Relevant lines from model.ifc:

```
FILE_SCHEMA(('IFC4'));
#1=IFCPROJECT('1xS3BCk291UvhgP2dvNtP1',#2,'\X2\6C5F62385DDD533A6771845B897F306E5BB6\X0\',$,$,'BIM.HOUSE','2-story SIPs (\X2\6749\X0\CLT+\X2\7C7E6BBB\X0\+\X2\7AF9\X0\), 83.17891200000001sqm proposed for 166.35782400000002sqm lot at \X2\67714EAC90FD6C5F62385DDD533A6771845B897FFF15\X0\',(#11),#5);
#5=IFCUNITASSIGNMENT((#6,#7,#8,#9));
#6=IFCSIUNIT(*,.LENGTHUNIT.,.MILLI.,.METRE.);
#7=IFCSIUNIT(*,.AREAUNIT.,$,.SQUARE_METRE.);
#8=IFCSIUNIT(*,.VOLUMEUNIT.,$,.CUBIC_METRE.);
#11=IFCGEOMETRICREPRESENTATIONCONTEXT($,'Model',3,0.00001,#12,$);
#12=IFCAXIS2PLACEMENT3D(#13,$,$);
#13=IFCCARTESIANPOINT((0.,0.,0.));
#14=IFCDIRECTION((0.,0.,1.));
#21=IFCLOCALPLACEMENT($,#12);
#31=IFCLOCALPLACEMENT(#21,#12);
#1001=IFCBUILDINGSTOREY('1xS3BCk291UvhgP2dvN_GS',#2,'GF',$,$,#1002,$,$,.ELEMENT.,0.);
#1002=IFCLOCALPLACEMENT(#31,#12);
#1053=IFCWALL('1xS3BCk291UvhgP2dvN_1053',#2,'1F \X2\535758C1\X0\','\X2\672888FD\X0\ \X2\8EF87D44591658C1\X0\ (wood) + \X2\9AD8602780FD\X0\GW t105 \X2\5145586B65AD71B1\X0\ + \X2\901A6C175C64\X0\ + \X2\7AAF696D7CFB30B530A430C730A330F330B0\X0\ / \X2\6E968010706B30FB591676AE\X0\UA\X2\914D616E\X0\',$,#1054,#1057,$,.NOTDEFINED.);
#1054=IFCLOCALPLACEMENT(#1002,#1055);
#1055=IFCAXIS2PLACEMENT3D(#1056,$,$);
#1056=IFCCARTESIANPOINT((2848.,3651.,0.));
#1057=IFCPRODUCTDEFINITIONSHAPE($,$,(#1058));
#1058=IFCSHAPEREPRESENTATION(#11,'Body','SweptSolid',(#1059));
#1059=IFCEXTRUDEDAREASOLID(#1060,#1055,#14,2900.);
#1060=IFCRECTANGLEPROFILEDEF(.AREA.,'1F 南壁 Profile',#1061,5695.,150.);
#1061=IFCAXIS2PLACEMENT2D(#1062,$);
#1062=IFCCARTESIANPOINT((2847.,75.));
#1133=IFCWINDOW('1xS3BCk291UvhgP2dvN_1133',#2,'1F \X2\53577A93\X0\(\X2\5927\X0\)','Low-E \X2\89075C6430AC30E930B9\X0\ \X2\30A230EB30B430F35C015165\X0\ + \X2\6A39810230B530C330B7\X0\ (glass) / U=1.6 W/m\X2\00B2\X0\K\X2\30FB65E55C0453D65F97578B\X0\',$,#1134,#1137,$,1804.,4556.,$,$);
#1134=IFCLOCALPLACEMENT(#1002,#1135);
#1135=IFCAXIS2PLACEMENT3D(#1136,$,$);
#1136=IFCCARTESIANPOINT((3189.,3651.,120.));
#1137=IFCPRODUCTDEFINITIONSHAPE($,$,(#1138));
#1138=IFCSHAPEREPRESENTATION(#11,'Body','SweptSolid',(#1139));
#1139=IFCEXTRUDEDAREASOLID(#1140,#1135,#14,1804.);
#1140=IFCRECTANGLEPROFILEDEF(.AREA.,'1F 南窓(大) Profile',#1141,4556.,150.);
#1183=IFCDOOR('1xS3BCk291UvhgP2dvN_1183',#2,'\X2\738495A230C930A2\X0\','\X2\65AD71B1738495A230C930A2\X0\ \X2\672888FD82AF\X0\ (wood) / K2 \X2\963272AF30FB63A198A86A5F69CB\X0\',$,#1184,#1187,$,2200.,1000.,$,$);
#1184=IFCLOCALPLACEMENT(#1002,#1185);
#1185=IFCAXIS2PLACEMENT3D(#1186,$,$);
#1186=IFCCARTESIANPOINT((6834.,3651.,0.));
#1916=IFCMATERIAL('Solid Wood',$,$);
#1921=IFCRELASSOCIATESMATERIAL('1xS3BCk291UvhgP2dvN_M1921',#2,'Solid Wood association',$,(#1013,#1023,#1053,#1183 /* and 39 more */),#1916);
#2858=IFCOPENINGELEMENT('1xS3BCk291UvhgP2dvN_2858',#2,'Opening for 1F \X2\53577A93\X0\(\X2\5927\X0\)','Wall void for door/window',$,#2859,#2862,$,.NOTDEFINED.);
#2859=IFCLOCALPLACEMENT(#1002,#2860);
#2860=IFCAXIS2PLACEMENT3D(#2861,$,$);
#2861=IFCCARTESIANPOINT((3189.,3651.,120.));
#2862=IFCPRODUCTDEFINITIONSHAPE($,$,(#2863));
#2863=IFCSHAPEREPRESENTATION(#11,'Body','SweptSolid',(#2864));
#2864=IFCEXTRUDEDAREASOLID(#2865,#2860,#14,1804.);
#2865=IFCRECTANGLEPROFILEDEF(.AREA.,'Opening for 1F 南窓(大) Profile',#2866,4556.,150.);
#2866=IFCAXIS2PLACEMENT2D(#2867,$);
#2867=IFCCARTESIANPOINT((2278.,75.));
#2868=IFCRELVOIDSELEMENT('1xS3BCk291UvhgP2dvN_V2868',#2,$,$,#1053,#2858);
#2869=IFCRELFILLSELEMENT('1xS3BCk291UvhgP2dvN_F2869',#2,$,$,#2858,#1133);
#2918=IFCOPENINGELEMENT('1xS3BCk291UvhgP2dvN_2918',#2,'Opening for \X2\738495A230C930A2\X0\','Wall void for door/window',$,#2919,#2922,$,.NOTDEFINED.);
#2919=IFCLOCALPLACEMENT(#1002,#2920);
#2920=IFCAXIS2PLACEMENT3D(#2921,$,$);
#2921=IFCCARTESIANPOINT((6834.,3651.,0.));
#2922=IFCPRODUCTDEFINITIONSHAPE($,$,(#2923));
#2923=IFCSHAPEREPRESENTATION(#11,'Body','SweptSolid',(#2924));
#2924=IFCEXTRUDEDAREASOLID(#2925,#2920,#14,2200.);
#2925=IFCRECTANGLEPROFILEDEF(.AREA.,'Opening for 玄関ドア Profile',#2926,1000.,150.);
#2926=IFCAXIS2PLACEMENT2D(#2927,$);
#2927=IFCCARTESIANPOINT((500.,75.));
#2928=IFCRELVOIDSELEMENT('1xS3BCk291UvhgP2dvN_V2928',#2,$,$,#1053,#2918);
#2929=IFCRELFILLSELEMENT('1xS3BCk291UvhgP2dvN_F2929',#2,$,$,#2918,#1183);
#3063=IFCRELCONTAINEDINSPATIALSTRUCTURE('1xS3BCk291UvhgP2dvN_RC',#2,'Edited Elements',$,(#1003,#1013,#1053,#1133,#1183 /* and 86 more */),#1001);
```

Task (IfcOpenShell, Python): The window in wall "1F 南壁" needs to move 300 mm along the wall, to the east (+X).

```python
import ifcopenshell
import ifcopenshell.api.geometry
import ifcopenshell.util.placement
import ifcopenshell.util.unit

model = ifcopenshell.open("model.ifc")
unit_scale = ifcopenshell.util.unit.calculate_unit_scale(model)

window = model.by_guid("1xS3BCk291UvhgP2dvN_1133")
opening = window.FillsVoids[0].RelatingOpeningElement
wall = opening.VoidsElements[0].RelatingBuildingElement

wall_matrix = ifcopenshell.util.placement.get_local_placement(wall.ObjectPlacement)
shift = wall_matrix[:3, 0] * 0.3 / unit_scale
before = ifcopenshell.util.placement.get_local_placement(window.ObjectPlacement)[:3, 3].copy()

# The window is not placed relative to its opening, so move both.
for product in (opening, window):
    matrix = ifcopenshell.util.placement.get_local_placement(product.ObjectPlacement)
    matrix[:3, 3] += shift
    ifcopenshell.api.geometry.edit_object_placement(model, product=product, matrix=matrix, is_si=False)

after = ifcopenshell.util.placement.get_local_placement(window.ObjectPlacement)[:3, 3]
print("window moved by", (after - before).round(3) + 0.0)

model.write("model_v2.ifc")
```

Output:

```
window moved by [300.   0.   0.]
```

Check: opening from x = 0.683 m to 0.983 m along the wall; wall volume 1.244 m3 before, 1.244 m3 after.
